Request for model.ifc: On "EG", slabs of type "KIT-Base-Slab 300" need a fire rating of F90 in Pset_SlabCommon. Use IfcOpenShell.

First a look at what the model holds.

```python
import ifcopenshell
import ifcopenshell.util.element

model = ifcopenshell.open("model.ifc")
print(model.schema)
storey = next(s for s in model.by_type("IfcBuildingStorey") if s.Name == "EG")
slabs = [e for e in ifcopenshell.util.element.get_decomposition(storey) if e.is_a("IfcSlab")]
seen = {}
for e in slabs:
    element_type = ifcopenshell.util.element.get_type(e)
    key = (element_type.Name if element_type != e and element_type else None, ifcopenshell.util.element.get_pset(e, "Pset_SlabCommon", "FireRating"))
    seen[key] = seen.get(key, 0) + 1
for (name, value), count in sorted(seen.items(), key=str):
    print(count, "x", name, "|", value)
```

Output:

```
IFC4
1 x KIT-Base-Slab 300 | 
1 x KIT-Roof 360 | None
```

```python
import ifcopenshell
import ifcopenshell.api.pset
import ifcopenshell.util.element

model = ifcopenshell.open("model.ifc")

storey = next(s for s in model.by_type("IfcBuildingStorey") if s.Name == "EG")
slabs = [e for e in ifcopenshell.util.element.get_decomposition(storey) if e.is_a("IfcSlab")]

count = 0
for e in slabs:
    element_type = ifcopenshell.util.element.get_type(e)
    if element_type in (None, e) or element_type.Name != "KIT-Base-Slab 300":
        continue
    # add_pset returns the element's existing set when there is one.
    pset = ifcopenshell.api.pset.add_pset(model, product=e, name="Pset_SlabCommon")
    ifcopenshell.api.pset.edit_pset(model, pset=pset, properties={"FireRating": "F90"})
    count += 1

print(count, "slabs updated")

model.write("model_updated.ifc")
```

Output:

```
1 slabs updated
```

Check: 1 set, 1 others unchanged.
